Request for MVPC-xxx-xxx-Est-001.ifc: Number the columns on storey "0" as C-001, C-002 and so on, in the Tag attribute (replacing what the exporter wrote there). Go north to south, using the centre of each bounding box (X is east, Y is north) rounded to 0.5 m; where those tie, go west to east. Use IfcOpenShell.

First a look at what the model holds.

```python
import ifcopenshell
import ifcopenshell.util.element
import ifcopenshell.util.placement

model = ifcopenshell.open("MVPC-xxx-xxx-Est-001.ifc")
print(model.schema)
storey = next(s for s in model.by_type("IfcBuildingStorey") if s.Name == "0")
columns = [e for e in ifcopenshell.util.element.get_decomposition(storey) if e.is_a("IfcColumn")]
for e in sorted(columns, key=lambda e: e.id()):
    origin = ifcopenshell.util.placement.get_local_placement(e.ObjectPlacement)[:3, 3]
    print(e.id(), e.Tag, e.Name, origin.round(2) + 0.0, sep=" | ")
```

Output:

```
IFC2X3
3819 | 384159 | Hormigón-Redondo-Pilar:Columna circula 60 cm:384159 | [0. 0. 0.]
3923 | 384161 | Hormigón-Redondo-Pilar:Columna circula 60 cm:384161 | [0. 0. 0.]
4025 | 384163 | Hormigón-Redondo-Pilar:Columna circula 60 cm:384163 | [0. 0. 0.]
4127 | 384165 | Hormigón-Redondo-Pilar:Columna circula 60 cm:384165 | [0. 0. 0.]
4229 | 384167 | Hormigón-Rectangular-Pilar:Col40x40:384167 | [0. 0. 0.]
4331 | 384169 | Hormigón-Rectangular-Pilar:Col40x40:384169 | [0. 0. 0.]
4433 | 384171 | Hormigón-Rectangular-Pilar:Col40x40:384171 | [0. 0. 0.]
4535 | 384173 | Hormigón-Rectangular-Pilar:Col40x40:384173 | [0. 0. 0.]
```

```python
import ifcopenshell
import ifcopenshell.geom
import ifcopenshell.util.element
import ifcopenshell.util.shape

model = ifcopenshell.open("MVPC-xxx-xxx-Est-001.ifc")
settings = ifcopenshell.geom.settings()
settings.set("use-world-coords", True)


def centre(element):
    shape = ifcopenshell.geom.create_shape(settings, element)
    return ifcopenshell.util.shape.get_bbox_centroid(shape.geometry)


storey = next(s for s in model.by_type("IfcBuildingStorey") if s.Name == "0")
columns = [e for e in ifcopenshell.util.element.get_decomposition(storey) if e.is_a("IfcColumn")]

# Insertion points can sit at a corner or the storey origin, so sort by the geometry (in metres).
centres = {e: centre(e) for e in columns}
columns.sort(key=lambda e: (-round(centres[e][1] / 0.5), centres[e][0]))

for i, e in enumerate(columns, start=1):
    number = f"C-0{i:02d}"
    e.Tag = number
    print(e.id(), number)

model.write("MVPC-xxx-xxx-Est-001-out.ifc")
```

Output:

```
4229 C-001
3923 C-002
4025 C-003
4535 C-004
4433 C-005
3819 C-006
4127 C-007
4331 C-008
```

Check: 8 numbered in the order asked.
